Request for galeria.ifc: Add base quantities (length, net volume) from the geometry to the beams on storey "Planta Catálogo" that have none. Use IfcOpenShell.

First a look at what the model holds.

```python
import ifcopenshell
import ifcopenshell.util.element
import ifcopenshell.util.unit

model = ifcopenshell.open("galeria.ifc")
print(model.schema)
for unit_type in ("LENGTHUNIT", "AREAUNIT", "VOLUMEUNIT"):
    print(unit_type, ifcopenshell.util.unit.calculate_unit_scale(model, unit_type))
storey = next(s for s in model.by_type("IfcBuildingStorey") if s.Name == "Planta Catálogo")
beams = [e for e in ifcopenshell.util.element.get_decomposition(storey) if e.is_a("IfcBeam")]
for e in sorted(beams, key=lambda e: e.id()):
    print(e.id(), e.is_a(), e.Name, list(ifcopenshell.util.element.get_psets(e, qtos_only=True)), sep=" | ")
```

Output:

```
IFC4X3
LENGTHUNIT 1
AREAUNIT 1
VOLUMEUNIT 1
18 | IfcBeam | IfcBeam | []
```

```python
import ifcopenshell
import ifcopenshell.api.pset
import ifcopenshell.geom
import ifcopenshell.util.element
import ifcopenshell.util.shape
import ifcopenshell.util.unit

model = ifcopenshell.open("galeria.ifc")
unit_scale = ifcopenshell.util.unit.calculate_unit_scale(model)
volume_scale = ifcopenshell.util.unit.calculate_unit_scale(model, "VOLUMEUNIT")
settings = ifcopenshell.geom.settings()

storey = next(s for s in model.by_type("IfcBuildingStorey") if s.Name == "Planta Catálogo")
beams = [e for e in ifcopenshell.util.element.get_decomposition(storey) if e.is_a("IfcBeam")]

for e in sorted(beams, key=lambda e: e.id()):
    if ifcopenshell.util.element.get_psets(e, qtos_only=True, should_inherit=False):
        continue
    # Geometry comes back in metres, in the element's own axes.
    shape = ifcopenshell.geom.create_shape(settings, e)
    values = {
        "Length": ifcopenshell.util.shape.get_max_xyz(shape.geometry) / unit_scale,
        "NetVolume": ifcopenshell.util.shape.get_volume(shape.geometry) / volume_scale,
    }
    qto = ifcopenshell.api.pset.add_qto(model, product=e, name="Qto_BeamBaseQuantities")
    ifcopenshell.api.pset.edit_qto(model, qto=qto, properties=values)
    print(e.id(), {k: round(v, 3) for k, v in values.items()})

model.write("galeria_rev.ifc")
```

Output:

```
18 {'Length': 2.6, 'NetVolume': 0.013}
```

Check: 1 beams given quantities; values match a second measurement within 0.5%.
